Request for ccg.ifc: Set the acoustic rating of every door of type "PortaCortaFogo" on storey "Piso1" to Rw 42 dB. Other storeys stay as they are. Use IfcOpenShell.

First a look at what the model holds.

```python
import ifcopenshell
import ifcopenshell.util.element

model = ifcopenshell.open("ccg.ifc")
print(model.schema)
storey = next(s for s in model.by_type("IfcBuildingStorey") if s.Name == "Piso1")
doors = [e for e in ifcopenshell.util.element.get_decomposition(storey) if e.is_a("IfcDoor")]
seen = {}
for e in doors:
    element_type = ifcopenshell.util.element.get_type(e)
    key = (element_type.Name if element_type != e and element_type else None, ifcopenshell.util.element.get_pset(e, "Pset_DoorCommon", "AcousticRating"))
    seen[key] = seen.get(key, 0) + 1
for (name, value), count in sorted(seen.items(), key=str):
    print(count, "x", name, "|", value)
```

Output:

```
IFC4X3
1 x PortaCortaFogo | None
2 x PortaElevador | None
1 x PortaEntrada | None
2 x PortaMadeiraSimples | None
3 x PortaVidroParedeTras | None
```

```python
import ifcopenshell
import ifcopenshell.api.pset
import ifcopenshell.util.element

model = ifcopenshell.open("ccg.ifc")

storey = next(s for s in model.by_type("IfcBuildingStorey") if s.Name == "Piso1")
doors = [e for e in ifcopenshell.util.element.get_decomposition(storey) if e.is_a("IfcDoor")]

count = 0
for e in doors:
    element_type = ifcopenshell.util.element.get_type(e)
    if element_type in (None, e) or element_type.Name != "PortaCortaFogo":
        continue
    # add_pset returns the element's existing set when there is one.
    pset = ifcopenshell.api.pset.add_pset(model, product=e, name="Pset_DoorCommon")
    ifcopenshell.api.pset.edit_pset(model, pset=pset, properties={"AcousticRating": "Rw 42 dB"})
    count += 1

print(count, "doors updated")

model.write("ccg_rev.ifc")
```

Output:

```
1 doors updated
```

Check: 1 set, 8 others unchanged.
